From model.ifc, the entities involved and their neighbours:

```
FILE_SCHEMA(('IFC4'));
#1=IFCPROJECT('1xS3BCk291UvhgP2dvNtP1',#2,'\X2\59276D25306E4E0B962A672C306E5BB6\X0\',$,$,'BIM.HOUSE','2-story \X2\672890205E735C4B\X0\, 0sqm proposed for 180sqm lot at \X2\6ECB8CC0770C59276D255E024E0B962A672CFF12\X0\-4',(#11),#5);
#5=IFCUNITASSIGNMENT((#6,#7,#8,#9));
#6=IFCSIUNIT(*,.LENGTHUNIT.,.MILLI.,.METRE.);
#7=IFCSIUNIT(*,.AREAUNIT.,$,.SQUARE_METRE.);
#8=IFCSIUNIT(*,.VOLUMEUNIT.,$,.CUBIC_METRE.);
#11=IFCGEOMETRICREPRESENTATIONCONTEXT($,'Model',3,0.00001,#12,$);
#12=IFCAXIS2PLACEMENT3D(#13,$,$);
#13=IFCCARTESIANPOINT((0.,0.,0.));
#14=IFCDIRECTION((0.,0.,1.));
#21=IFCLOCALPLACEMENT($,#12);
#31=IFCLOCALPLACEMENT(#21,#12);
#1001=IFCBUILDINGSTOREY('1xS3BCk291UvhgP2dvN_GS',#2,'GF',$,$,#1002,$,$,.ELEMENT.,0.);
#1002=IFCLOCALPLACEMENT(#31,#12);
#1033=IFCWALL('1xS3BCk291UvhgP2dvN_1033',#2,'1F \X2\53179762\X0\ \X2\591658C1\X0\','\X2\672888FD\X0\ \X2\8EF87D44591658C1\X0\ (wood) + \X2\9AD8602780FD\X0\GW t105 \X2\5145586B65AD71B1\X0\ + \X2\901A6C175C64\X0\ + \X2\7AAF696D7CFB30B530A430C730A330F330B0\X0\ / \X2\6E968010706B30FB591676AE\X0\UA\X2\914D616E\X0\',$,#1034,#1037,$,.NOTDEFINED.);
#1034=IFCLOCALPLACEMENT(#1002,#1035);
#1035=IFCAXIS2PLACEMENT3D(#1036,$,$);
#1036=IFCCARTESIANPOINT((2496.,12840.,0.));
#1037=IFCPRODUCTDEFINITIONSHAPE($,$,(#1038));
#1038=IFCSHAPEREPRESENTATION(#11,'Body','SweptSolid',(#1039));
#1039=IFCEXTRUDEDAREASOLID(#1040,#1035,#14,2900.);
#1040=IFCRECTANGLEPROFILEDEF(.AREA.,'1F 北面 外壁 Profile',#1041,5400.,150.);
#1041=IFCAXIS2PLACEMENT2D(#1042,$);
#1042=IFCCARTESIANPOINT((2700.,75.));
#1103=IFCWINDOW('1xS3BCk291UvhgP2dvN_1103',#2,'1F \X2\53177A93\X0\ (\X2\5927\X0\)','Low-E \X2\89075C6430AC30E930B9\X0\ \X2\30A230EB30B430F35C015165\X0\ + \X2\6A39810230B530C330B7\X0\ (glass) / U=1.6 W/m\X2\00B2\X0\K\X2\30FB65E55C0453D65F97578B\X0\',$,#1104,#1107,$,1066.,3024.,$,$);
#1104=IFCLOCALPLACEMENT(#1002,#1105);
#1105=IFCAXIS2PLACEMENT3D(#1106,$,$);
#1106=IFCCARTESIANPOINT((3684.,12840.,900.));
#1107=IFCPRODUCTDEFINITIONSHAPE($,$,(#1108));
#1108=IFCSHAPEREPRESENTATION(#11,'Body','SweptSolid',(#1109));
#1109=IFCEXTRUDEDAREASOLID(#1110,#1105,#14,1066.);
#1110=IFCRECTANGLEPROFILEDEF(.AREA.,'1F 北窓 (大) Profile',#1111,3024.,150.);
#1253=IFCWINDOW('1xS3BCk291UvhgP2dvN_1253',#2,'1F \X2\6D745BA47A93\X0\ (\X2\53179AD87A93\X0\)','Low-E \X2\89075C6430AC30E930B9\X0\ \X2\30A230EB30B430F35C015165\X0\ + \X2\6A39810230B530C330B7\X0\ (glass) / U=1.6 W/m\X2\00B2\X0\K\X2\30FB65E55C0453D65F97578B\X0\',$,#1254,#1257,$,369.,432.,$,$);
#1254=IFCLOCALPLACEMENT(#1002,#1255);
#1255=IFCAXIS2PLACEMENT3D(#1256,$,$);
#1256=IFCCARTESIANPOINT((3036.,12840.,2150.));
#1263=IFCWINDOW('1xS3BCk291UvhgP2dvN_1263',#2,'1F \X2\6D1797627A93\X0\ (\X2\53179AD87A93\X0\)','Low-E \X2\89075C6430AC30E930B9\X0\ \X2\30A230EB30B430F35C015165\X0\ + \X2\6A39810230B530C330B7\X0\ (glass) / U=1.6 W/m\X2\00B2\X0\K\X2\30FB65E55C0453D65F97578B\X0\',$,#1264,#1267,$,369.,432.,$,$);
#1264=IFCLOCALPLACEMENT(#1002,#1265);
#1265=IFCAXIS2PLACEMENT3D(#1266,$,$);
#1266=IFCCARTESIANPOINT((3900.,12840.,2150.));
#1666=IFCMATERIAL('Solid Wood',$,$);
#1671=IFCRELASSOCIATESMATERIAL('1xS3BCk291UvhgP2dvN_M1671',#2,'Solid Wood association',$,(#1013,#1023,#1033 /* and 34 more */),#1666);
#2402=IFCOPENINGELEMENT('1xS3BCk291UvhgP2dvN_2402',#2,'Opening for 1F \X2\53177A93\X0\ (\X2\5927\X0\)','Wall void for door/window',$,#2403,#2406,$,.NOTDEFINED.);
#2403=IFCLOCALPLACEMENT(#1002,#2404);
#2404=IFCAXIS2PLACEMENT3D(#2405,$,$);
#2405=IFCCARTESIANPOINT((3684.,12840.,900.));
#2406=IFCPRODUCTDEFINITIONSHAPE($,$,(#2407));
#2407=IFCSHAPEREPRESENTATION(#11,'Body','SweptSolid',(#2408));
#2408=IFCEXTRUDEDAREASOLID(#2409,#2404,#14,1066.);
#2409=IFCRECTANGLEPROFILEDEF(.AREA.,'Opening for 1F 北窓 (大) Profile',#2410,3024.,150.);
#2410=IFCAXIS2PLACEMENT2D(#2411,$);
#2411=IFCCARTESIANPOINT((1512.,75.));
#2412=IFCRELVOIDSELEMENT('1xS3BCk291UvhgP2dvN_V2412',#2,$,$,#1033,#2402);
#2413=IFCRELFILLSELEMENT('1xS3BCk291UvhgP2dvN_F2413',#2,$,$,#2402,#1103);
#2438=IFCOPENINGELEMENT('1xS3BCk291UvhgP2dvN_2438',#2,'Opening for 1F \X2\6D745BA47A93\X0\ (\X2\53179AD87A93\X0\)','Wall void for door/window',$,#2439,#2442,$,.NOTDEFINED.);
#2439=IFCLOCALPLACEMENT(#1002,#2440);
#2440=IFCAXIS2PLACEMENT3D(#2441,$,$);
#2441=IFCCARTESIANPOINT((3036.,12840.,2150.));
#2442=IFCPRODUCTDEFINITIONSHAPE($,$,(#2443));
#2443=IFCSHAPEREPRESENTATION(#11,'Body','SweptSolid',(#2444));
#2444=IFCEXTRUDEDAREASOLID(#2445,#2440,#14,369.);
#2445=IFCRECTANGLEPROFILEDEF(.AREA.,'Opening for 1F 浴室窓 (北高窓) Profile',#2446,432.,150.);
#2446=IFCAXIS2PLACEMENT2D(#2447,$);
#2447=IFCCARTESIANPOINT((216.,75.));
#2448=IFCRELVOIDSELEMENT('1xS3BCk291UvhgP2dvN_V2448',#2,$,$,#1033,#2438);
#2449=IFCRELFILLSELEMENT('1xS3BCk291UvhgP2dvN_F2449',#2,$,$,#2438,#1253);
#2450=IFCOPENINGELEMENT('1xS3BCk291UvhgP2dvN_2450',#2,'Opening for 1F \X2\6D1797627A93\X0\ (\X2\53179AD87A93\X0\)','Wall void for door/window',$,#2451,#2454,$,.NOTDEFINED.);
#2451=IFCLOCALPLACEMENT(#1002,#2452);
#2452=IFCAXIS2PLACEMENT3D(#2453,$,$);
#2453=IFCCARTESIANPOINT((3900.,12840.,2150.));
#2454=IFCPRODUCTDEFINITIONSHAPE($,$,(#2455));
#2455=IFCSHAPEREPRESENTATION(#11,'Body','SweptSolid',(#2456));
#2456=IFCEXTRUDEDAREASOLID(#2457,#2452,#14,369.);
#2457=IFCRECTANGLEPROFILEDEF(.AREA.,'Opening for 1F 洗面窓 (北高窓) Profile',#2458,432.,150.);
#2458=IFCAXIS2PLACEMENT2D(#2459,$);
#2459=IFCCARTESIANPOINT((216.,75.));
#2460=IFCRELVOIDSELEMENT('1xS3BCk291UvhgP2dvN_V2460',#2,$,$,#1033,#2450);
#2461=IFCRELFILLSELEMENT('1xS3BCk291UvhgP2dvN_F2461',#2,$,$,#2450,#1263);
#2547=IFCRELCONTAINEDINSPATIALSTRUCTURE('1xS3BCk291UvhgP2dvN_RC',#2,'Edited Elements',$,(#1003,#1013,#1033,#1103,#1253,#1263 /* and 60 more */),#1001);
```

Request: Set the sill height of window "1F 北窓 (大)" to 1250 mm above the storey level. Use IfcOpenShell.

```python
import numpy as np
import ifcopenshell
import ifcopenshell.api.geometry
import ifcopenshell.geom
import ifcopenshell.util.element
import ifcopenshell.util.placement
import ifcopenshell.util.shape
import ifcopenshell.util.unit

model = ifcopenshell.open("model.ifc")
unit_scale = ifcopenshell.util.unit.calculate_unit_scale(model)

window = model.by_guid("1xS3BCk291UvhgP2dvN_1103")
opening = window.FillsVoids[0].RelatingOpeningElement
storey = ifcopenshell.util.element.get_container(window, ifc_class="IfcBuildingStorey")
level = ifcopenshell.util.placement.get_local_placement(storey.ObjectPlacement)[2, 3]

# The opening's origin need not be at the sill, so measure its lowest point.
shape = ifcopenshell.geom.create_shape(ifcopenshell.geom.settings(), opening)
bottom = ifcopenshell.util.shape.get_shape_bottom_elevation(shape, shape.geometry) / unit_scale
dz = level + 1.25 / unit_scale - bottom

shift = np.array([0.0, 0.0, dz])
# The window is not placed relative to its opening, so move both.
for product in (opening, window):
    matrix = ifcopenshell.util.placement.get_local_placement(product.ObjectPlacement)
    matrix[:3, 3] += shift
    ifcopenshell.api.geometry.edit_object_placement(model, product=product, matrix=matrix, is_si=False)

print(f"moved by {dz * unit_scale:+.3f} m")

model.write("model_updated.ifc")
```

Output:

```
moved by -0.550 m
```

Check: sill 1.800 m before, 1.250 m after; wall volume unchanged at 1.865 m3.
